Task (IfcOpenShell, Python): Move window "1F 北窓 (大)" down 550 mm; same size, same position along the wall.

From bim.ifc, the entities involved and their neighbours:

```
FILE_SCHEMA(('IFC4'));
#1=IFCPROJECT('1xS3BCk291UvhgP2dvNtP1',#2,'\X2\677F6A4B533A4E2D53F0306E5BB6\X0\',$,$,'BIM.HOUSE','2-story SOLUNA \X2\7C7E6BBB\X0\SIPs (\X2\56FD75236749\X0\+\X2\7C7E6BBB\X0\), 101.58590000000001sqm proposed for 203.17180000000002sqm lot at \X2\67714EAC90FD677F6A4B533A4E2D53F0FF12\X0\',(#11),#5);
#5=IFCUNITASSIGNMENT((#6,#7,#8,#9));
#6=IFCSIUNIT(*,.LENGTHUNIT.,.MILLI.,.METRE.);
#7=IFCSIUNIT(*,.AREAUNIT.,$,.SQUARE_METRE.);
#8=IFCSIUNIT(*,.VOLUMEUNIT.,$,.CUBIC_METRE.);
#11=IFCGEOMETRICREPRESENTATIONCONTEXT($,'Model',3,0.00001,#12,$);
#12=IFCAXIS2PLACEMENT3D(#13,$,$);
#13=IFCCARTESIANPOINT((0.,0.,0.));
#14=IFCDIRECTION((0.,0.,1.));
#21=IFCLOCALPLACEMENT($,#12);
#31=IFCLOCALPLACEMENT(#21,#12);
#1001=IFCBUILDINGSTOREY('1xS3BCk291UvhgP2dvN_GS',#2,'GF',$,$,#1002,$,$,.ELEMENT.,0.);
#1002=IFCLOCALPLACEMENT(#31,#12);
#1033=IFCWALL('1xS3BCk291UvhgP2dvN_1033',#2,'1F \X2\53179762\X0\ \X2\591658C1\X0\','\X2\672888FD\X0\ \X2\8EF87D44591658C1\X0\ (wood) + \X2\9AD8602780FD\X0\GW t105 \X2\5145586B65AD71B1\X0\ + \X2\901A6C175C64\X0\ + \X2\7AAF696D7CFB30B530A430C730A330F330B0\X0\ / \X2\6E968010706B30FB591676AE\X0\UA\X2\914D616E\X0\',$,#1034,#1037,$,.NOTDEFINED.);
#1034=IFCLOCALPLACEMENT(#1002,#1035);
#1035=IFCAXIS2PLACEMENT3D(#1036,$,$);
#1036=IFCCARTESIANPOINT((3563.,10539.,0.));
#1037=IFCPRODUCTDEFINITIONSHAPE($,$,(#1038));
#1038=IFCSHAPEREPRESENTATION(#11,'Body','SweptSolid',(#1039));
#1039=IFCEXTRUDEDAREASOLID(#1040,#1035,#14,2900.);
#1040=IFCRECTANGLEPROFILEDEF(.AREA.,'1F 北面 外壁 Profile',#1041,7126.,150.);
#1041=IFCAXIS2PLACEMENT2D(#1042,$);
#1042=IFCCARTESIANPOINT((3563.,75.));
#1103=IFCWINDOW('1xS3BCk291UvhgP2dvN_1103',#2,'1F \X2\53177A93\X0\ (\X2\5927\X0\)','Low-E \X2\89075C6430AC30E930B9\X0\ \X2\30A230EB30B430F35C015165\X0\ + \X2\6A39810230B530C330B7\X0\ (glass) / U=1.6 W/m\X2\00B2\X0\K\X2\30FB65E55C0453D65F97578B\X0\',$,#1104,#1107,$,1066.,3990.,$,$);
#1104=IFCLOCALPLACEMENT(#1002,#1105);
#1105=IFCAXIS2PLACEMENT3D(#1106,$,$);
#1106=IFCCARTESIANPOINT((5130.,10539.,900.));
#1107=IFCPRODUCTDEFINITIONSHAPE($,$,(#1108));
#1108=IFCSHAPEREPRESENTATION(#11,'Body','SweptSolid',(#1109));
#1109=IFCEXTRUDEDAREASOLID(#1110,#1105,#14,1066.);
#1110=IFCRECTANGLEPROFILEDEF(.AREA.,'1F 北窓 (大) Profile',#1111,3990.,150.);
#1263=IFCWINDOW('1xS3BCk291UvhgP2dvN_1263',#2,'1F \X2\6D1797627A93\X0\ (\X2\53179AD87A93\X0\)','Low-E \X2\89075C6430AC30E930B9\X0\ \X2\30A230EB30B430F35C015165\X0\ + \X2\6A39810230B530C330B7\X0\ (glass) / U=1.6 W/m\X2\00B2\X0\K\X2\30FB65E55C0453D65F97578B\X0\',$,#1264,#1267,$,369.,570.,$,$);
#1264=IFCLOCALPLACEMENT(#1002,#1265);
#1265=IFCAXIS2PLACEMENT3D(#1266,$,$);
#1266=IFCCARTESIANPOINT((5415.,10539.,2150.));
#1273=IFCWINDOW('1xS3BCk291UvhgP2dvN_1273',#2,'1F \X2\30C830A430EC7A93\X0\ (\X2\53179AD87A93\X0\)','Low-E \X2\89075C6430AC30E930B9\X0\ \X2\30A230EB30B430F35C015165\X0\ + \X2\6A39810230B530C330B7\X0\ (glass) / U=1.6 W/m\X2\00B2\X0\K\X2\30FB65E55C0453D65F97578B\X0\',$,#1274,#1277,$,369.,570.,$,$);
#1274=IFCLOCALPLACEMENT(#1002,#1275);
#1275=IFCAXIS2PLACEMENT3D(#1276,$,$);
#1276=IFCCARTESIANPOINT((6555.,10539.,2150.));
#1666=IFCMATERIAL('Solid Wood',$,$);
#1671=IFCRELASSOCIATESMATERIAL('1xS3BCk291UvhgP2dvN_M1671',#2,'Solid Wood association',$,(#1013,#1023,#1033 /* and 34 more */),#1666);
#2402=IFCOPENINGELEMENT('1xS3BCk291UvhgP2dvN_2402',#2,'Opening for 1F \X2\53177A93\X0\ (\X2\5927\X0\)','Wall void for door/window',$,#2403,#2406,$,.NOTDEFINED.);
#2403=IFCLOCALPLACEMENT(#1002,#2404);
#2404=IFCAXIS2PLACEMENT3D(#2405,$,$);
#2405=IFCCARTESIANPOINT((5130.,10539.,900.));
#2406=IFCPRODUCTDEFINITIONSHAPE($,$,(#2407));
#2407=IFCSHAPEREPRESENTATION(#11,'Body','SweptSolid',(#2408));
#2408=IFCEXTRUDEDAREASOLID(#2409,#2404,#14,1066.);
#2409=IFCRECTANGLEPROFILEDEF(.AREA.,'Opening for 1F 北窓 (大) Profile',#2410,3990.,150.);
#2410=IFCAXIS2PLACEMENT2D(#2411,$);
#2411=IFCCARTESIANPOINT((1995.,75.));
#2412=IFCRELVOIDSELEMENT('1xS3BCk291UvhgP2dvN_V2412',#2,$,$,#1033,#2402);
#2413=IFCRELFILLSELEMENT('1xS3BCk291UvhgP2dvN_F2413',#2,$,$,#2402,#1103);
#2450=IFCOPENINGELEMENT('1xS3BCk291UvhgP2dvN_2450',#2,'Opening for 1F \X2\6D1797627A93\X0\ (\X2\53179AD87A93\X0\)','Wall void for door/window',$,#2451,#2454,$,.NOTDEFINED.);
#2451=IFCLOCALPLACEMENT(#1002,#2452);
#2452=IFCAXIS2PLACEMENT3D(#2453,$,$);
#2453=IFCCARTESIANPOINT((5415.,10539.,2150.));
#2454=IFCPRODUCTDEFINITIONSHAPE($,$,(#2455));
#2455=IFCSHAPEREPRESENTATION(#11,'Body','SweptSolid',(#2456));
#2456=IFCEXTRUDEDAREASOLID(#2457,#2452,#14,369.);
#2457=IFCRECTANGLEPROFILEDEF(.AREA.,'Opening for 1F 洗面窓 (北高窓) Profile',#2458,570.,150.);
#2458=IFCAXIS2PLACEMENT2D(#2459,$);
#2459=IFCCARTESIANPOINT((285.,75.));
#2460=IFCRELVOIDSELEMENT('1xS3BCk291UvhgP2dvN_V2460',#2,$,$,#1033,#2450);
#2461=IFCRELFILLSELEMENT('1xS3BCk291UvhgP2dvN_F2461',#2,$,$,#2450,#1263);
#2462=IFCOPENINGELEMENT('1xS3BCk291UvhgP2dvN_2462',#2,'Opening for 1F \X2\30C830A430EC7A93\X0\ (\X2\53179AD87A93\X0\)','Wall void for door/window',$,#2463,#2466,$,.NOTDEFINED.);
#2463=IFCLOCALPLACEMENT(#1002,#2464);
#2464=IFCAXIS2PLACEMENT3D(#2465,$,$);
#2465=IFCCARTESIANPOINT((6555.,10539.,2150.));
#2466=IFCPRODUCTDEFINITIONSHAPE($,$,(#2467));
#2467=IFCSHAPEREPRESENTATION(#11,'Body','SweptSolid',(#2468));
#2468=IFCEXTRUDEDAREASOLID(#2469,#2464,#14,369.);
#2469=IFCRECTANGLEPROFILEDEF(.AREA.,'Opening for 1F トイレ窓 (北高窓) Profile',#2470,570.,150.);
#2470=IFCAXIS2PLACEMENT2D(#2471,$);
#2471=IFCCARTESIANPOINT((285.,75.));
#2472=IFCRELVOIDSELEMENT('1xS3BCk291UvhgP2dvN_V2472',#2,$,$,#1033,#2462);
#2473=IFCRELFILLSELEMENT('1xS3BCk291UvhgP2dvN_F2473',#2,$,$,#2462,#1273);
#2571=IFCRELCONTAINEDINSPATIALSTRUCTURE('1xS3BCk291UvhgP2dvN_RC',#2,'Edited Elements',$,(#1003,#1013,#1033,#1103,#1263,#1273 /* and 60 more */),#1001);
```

```python
import numpy as np
import ifcopenshell
import ifcopenshell.api.geometry
import ifcopenshell.util.placement
import ifcopenshell.util.unit

model = ifcopenshell.open("bim.ifc")
unit_scale = ifcopenshell.util.unit.calculate_unit_scale(model)

window = model.by_id(1103)
opening = window.FillsVoids[0].RelatingOpeningElement
dz = -0.55 / unit_scale

shift = np.array([0.0, 0.0, dz])
# The window is not placed relative to its opening, so move both.
for product in (opening, window):
    matrix = ifcopenshell.util.placement.get_local_placement(product.ObjectPlacement)
    matrix[:3, 3] += shift
    ifcopenshell.api.geometry.edit_object_placement(model, product=product, matrix=matrix, is_si=False)

print(f"moved by {dz * unit_scale:+.3f} m")

model.write("bim-out.ifc")
```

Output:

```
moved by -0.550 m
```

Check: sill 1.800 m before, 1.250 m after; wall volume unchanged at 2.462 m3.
